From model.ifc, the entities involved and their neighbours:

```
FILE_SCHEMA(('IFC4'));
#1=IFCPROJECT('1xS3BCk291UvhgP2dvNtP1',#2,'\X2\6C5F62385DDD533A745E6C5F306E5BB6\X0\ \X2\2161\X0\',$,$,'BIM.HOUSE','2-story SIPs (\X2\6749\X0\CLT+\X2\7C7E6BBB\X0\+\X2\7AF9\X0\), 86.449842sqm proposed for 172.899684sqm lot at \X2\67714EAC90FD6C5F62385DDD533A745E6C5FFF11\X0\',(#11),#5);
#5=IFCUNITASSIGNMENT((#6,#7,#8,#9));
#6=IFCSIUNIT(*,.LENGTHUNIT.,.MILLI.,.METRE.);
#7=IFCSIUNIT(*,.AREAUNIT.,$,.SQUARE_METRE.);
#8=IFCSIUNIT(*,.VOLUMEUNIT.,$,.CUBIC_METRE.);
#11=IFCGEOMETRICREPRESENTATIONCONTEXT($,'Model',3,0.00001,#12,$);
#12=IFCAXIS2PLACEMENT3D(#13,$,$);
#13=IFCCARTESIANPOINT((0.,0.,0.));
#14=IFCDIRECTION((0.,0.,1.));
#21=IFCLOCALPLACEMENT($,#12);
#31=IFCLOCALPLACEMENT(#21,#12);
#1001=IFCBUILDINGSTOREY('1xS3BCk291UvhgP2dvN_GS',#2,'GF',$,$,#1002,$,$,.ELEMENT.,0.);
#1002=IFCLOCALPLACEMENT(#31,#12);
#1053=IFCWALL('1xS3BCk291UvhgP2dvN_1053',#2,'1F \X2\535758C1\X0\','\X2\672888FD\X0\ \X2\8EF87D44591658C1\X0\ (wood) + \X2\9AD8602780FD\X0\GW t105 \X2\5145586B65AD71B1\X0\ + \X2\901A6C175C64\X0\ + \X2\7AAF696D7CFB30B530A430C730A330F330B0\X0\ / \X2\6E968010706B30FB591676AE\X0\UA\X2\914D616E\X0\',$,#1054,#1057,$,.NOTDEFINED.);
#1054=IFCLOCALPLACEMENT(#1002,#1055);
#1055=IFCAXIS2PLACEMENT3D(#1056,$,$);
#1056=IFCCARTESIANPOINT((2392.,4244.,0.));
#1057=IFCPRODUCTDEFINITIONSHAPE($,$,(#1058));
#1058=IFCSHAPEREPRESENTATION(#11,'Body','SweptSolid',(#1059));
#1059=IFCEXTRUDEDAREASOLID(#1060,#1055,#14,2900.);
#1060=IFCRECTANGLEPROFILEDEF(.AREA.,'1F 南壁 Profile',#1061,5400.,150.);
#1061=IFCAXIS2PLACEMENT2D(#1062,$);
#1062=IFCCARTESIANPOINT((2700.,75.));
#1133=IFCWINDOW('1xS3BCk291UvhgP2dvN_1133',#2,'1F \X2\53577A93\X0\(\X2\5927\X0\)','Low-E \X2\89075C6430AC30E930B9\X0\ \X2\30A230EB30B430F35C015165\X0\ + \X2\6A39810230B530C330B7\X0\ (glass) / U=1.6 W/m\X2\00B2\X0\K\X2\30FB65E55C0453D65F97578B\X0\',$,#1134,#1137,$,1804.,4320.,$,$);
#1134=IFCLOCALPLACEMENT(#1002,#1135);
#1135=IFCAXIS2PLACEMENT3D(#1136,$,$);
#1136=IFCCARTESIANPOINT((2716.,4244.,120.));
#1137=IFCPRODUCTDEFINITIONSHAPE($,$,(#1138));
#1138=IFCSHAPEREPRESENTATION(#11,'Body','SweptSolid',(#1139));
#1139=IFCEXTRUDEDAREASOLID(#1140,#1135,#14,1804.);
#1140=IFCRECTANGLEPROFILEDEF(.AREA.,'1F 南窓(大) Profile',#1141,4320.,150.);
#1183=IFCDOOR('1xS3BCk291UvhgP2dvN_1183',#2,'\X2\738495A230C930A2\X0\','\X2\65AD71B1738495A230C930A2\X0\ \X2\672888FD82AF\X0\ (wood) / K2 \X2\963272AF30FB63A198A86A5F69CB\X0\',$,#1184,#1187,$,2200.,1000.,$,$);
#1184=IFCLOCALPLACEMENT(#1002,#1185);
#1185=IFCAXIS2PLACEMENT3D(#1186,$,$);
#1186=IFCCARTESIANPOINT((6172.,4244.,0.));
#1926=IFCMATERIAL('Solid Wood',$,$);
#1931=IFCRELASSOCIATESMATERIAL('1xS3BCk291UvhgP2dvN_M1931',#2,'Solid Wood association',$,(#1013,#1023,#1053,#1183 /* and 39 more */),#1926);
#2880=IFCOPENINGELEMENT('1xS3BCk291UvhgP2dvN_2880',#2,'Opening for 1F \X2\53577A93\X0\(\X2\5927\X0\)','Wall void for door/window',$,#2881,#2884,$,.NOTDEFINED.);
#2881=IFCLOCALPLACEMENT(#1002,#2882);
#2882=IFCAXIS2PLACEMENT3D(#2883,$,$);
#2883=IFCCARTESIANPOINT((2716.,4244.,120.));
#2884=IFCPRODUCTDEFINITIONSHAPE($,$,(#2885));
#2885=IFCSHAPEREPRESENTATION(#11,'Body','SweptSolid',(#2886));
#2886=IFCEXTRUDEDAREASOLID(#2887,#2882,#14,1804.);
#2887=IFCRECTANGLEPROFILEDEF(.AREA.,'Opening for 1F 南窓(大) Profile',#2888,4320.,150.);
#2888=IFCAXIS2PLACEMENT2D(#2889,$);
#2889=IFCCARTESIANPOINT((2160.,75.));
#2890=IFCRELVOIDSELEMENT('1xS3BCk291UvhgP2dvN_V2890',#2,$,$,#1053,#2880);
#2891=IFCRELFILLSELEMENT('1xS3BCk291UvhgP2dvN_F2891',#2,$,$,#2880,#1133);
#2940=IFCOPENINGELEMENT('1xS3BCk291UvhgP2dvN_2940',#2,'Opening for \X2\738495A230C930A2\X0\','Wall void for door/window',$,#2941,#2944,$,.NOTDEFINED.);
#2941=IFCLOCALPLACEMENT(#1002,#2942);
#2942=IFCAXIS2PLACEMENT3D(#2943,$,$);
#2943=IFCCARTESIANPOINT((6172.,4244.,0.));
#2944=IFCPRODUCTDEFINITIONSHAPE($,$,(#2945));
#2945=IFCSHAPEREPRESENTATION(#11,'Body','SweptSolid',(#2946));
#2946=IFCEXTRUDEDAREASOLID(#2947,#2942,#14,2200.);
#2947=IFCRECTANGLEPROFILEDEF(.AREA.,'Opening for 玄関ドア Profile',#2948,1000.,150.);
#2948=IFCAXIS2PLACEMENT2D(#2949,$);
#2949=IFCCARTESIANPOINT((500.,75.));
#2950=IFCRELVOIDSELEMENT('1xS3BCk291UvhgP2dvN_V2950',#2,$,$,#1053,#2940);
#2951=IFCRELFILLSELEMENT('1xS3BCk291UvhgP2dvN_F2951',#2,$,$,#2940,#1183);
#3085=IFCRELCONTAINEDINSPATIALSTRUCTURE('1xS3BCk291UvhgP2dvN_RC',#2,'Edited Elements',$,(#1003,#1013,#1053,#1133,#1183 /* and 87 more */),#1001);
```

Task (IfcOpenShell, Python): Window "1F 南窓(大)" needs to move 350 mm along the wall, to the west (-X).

```python
import ifcopenshell
import ifcopenshell.api.geometry
import ifcopenshell.util.placement

model = ifcopenshell.open("model.ifc")

window = model.by_id(1133)
opening = window.FillsVoids[0].RelatingOpeningElement
wall = opening.VoidsElements[0].RelatingBuildingElement

wall_matrix = ifcopenshell.util.placement.get_local_placement(wall.ObjectPlacement)
shift = wall_matrix[:3, 0] * -350.0
before = ifcopenshell.util.placement.get_local_placement(window.ObjectPlacement)[:3, 3].copy()

# The window is not placed relative to its opening, so move both.
for product in (opening, window):
    matrix = ifcopenshell.util.placement.get_local_placement(product.ObjectPlacement)
    matrix[:3, 3] += shift
    ifcopenshell.api.geometry.edit_object_placement(model, product=product, matrix=matrix, is_si=False)

after = ifcopenshell.util.placement.get_local_placement(window.ObjectPlacement)[:3, 3]
print("window moved by", (after - before).round(3) + 0.0)

model.write("model-out.ifc")
```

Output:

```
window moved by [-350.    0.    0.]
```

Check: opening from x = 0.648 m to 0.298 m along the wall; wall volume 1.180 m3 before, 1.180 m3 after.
